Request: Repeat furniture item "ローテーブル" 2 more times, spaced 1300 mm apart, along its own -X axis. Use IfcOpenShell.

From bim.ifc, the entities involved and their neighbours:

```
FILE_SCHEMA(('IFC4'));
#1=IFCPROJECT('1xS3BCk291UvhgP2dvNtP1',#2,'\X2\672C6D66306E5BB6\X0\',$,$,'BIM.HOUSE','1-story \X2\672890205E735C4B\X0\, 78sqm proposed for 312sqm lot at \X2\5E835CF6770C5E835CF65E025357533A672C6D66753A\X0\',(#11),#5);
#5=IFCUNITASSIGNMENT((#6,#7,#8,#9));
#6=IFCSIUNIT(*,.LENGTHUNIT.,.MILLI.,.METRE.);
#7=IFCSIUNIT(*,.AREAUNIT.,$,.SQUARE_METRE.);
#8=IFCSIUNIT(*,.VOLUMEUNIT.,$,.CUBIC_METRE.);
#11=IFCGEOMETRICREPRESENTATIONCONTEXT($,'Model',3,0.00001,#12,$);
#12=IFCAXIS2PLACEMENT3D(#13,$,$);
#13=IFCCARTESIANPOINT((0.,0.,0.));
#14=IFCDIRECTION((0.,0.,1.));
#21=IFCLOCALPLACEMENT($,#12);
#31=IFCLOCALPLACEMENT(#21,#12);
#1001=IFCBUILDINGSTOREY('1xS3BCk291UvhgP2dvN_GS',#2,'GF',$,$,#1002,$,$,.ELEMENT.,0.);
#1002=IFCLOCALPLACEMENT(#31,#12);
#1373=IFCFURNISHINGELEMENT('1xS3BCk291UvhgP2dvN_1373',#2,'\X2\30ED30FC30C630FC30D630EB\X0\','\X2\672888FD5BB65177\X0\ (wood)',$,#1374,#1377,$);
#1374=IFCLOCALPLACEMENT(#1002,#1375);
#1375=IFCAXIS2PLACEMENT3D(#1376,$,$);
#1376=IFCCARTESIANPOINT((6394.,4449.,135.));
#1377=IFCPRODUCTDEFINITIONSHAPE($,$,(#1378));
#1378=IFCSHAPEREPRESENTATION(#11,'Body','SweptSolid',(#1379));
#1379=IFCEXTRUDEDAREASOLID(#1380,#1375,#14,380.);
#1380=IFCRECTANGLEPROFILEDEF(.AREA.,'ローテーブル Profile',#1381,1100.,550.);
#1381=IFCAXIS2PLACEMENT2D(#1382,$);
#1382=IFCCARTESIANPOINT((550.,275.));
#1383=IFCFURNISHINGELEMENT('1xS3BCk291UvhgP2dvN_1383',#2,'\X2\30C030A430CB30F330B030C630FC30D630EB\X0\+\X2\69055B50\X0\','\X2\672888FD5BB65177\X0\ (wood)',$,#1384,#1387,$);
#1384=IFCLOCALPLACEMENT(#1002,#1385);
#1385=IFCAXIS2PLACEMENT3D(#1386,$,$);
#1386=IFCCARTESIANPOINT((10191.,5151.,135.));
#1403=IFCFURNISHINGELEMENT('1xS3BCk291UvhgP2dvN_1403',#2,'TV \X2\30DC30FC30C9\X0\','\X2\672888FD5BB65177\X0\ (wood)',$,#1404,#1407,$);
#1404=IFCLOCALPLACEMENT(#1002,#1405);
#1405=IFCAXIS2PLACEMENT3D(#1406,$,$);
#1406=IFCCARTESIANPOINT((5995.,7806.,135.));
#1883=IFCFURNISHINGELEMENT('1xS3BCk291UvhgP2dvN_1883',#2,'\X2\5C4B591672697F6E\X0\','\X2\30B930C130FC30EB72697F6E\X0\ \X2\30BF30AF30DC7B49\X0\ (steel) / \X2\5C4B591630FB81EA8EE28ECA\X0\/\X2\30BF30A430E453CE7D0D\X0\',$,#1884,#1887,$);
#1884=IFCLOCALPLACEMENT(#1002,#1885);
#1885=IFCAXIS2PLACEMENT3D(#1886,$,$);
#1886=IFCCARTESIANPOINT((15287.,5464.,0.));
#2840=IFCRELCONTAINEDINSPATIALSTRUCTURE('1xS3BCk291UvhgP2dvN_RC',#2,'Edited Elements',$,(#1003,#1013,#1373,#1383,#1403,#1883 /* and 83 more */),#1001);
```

```python
import ifcopenshell
import ifcopenshell.api.geometry
import ifcopenshell.api.root
import ifcopenshell.util.element
import ifcopenshell.util.placement
import ifcopenshell.util.unit

model = ifcopenshell.open("bim.ifc")
unit_scale = ifcopenshell.util.unit.calculate_unit_scale(model)


def reuse_history(source, copy):
    """copy_class also copies each property set's owner history, people and application; keep the originals."""
    for rel in copy.IsDefinedBy:
        if rel.is_a("IfcRelDefinesByProperties") and (history := rel.RelatingPropertyDefinition.OwnerHistory):
            rel.RelatingPropertyDefinition.OwnerHistory = source.OwnerHistory
            ifcopenshell.util.element.remove_deep2(model, history)


source = model.by_guid("1xS3BCk291UvhgP2dvN_1373")
base = ifcopenshell.util.placement.get_local_placement(source.ObjectPlacement)
step = -base[:3, 0] * 1.3 / unit_scale

for i in range(1, 3):
    copy = ifcopenshell.api.root.copy_class(model, product=source)
    copy.Representation = ifcopenshell.util.element.copy_deep(
        model, source.Representation, exclude=["IfcGeometricRepresentationContext", "IfcRepresentationMap"]
    )
    reuse_history(source, copy)
    matrix = base.copy()
    matrix[:3, 3] += i * step
    print("added at", matrix[:3, 3].round(3) + 0.0)
    ifcopenshell.api.geometry.edit_object_placement(model, product=copy, matrix=matrix, is_si=False)

model.write("bim_v2.ifc")
```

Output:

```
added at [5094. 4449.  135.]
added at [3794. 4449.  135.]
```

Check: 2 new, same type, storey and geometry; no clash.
